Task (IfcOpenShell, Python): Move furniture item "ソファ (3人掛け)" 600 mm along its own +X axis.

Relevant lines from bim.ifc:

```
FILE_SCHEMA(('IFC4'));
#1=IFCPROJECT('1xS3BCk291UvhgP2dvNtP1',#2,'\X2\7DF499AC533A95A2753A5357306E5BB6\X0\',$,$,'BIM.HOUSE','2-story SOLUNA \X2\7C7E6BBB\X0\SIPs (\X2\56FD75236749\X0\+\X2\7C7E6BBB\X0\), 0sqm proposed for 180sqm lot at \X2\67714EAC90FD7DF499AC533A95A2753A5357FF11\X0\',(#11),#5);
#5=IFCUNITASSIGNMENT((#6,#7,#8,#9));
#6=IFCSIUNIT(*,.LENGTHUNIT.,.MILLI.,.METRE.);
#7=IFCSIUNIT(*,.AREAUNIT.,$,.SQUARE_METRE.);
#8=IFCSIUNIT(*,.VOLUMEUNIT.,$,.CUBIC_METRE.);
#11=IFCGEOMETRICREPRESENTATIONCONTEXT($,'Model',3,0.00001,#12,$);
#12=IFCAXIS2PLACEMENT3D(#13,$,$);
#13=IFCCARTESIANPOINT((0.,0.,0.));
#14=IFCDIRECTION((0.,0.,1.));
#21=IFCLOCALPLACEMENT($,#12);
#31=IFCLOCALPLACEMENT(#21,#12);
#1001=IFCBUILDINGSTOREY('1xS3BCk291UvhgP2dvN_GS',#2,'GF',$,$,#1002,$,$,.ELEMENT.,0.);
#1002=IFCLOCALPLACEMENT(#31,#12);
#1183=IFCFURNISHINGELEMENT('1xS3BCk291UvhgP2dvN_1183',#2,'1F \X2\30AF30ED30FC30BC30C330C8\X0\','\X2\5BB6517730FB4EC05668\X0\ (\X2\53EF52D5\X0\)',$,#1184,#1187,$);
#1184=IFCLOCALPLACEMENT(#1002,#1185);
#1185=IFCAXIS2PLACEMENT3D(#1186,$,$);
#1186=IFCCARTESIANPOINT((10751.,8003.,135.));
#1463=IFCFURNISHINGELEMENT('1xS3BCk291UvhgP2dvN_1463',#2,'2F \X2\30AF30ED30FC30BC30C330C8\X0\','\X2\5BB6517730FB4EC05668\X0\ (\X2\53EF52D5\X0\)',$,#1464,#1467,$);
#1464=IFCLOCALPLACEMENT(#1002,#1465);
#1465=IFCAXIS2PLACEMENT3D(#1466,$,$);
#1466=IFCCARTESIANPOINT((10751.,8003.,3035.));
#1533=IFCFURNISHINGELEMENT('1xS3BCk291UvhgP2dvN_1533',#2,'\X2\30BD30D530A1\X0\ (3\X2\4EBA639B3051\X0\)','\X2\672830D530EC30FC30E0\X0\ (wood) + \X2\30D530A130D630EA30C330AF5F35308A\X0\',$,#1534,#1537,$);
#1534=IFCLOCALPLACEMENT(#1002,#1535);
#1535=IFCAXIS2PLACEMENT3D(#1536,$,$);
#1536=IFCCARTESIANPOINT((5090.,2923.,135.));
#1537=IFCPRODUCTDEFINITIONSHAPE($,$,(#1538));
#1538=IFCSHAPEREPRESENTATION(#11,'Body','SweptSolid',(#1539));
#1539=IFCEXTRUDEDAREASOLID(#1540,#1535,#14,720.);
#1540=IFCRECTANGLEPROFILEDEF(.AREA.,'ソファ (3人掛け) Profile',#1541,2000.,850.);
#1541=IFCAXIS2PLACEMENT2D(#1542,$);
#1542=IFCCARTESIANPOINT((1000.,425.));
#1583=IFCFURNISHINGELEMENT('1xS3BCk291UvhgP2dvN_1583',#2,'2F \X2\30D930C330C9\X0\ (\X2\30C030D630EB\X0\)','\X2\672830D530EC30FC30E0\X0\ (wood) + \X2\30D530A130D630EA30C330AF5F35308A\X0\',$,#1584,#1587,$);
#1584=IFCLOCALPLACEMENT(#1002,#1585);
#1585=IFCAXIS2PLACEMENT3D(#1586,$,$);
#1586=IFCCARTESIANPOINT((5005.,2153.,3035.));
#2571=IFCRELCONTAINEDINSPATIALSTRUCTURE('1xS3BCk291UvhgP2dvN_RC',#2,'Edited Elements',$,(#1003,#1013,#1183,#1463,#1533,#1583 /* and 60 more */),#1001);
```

```python
import ifcopenshell
import ifcopenshell.api.geometry
import ifcopenshell.util.placement

model = ifcopenshell.open("bim.ifc")

item = model.by_id(1533)
matrix = ifcopenshell.util.placement.get_local_placement(item.ObjectPlacement)
matrix[:3, 3] += matrix[:3, 0] * 600.0
ifcopenshell.api.geometry.edit_object_placement(model, product=item, matrix=matrix, is_si=False)

print(ifcopenshell.util.placement.get_local_placement(item.ObjectPlacement).round(3) + 0.0)

model.write("bim_rev.ifc")
```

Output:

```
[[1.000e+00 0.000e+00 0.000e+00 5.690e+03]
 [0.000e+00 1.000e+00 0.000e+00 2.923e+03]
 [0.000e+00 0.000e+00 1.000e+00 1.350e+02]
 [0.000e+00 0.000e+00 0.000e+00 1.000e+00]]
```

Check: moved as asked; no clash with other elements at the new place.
